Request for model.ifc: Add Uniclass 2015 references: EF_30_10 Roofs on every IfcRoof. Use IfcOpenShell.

First a look at what the model holds.

```python
import ifcopenshell

model = ifcopenshell.open("model.ifc")
print(model.schema)
print("classifications:", [c.Name for c in model.by_type("IfcClassification")])
for ifc_class in ("IfcDoor", "IfcRoof", "IfcStair", "IfcWall", "IfcWindow"):
    print(ifc_class, len(model.by_type(ifc_class)))
```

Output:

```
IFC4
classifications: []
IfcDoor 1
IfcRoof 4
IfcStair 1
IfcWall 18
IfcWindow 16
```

```python
import ifcopenshell
import ifcopenshell.api.classification

model = ifcopenshell.open("model.ifc")

system = ifcopenshell.api.classification.add_classification(model, classification="Uniclass 2015")

codes = {
    "IfcRoof": ("EF_30_10", "Roofs"),
}
for ifc_class, (code, name) in codes.items():
    products = model.by_type(ifc_class)
    ifcopenshell.api.classification.add_reference(
        model, products=products, classification=system, identification=code, name=name
    )
    print(code, len(products))

model.write("model_rev.ifc")
```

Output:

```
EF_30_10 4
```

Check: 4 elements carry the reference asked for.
